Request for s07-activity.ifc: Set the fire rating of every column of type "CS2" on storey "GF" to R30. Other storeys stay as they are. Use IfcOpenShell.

First a look at what the model holds.

```python
import ifcopenshell
import ifcopenshell.util.element

model = ifcopenshell.open("s07-activity.ifc")
print(model.schema)
storey = next(s for s in model.by_type("IfcBuildingStorey") if s.Name == "GF")
columns = [e for e in ifcopenshell.util.element.get_decomposition(storey) if e.is_a("IfcColumn")]
seen = {}
for e in columns:
    element_type = ifcopenshell.util.element.get_type(e)
    key = (element_type.Name if element_type != e and element_type else None, ifcopenshell.util.element.get_pset(e, "Pset_ColumnCommon", "FireRating"))
    seen[key] = seen.get(key, 0) + 1
for (name, value), count in sorted(seen.items(), key=str):
    print(count, "x", name, "|", value)
```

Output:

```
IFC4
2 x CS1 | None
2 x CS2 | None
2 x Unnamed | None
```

```python
import ifcopenshell
import ifcopenshell.api.pset
import ifcopenshell.util.element

model = ifcopenshell.open("s07-activity.ifc")

storey = next(s for s in model.by_type("IfcBuildingStorey") if s.Name == "GF")
columns = [e for e in ifcopenshell.util.element.get_decomposition(storey) if e.is_a("IfcColumn")]

count = 0
for e in columns:
    element_type = ifcopenshell.util.element.get_type(e)
    if element_type in (None, e) or element_type.Name != "CS2":
        continue
    # add_pset returns the element's existing set when there is one.
    pset = ifcopenshell.api.pset.add_pset(model, product=e, name="Pset_ColumnCommon")
    ifcopenshell.api.pset.edit_pset(model, pset=pset, properties={"FireRating": "R30"})
    count += 1

print(count, "columns updated")

model.write("s07-activity-out.ifc")
```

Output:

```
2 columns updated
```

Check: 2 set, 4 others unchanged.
